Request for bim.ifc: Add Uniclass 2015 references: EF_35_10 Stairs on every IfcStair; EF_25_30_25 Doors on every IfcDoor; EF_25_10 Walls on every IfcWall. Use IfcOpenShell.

First a look at what the model holds.

```python
import ifcopenshell

model = ifcopenshell.open("bim.ifc")
print(model.schema)
print("classifications:", [c.Name for c in model.by_type("IfcClassification")])
for ifc_class in ("IfcDoor", "IfcRoof", "IfcStair", "IfcWall", "IfcWindow"):
    print(ifc_class, len(model.by_type(ifc_class)))
```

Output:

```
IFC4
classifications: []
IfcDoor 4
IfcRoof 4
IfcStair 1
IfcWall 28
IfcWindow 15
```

```python
import ifcopenshell
import ifcopenshell.api.classification

model = ifcopenshell.open("bim.ifc")

system = ifcopenshell.api.classification.add_classification(model, classification="Uniclass 2015")

codes = {
    "IfcStair": ("EF_35_10", "Stairs"),
    "IfcDoor": ("EF_25_30_25", "Doors"),
    "IfcWall": ("EF_25_10", "Walls"),
}
for ifc_class, (code, name) in codes.items():
    products = model.by_type(ifc_class)
    ifcopenshell.api.classification.add_reference(
        model, products=products, classification=system, identification=code, name=name
    )
    print(code, len(products))

model.write("bim_rev.ifc")
```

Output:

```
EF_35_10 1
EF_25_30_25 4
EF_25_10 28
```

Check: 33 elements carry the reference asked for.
